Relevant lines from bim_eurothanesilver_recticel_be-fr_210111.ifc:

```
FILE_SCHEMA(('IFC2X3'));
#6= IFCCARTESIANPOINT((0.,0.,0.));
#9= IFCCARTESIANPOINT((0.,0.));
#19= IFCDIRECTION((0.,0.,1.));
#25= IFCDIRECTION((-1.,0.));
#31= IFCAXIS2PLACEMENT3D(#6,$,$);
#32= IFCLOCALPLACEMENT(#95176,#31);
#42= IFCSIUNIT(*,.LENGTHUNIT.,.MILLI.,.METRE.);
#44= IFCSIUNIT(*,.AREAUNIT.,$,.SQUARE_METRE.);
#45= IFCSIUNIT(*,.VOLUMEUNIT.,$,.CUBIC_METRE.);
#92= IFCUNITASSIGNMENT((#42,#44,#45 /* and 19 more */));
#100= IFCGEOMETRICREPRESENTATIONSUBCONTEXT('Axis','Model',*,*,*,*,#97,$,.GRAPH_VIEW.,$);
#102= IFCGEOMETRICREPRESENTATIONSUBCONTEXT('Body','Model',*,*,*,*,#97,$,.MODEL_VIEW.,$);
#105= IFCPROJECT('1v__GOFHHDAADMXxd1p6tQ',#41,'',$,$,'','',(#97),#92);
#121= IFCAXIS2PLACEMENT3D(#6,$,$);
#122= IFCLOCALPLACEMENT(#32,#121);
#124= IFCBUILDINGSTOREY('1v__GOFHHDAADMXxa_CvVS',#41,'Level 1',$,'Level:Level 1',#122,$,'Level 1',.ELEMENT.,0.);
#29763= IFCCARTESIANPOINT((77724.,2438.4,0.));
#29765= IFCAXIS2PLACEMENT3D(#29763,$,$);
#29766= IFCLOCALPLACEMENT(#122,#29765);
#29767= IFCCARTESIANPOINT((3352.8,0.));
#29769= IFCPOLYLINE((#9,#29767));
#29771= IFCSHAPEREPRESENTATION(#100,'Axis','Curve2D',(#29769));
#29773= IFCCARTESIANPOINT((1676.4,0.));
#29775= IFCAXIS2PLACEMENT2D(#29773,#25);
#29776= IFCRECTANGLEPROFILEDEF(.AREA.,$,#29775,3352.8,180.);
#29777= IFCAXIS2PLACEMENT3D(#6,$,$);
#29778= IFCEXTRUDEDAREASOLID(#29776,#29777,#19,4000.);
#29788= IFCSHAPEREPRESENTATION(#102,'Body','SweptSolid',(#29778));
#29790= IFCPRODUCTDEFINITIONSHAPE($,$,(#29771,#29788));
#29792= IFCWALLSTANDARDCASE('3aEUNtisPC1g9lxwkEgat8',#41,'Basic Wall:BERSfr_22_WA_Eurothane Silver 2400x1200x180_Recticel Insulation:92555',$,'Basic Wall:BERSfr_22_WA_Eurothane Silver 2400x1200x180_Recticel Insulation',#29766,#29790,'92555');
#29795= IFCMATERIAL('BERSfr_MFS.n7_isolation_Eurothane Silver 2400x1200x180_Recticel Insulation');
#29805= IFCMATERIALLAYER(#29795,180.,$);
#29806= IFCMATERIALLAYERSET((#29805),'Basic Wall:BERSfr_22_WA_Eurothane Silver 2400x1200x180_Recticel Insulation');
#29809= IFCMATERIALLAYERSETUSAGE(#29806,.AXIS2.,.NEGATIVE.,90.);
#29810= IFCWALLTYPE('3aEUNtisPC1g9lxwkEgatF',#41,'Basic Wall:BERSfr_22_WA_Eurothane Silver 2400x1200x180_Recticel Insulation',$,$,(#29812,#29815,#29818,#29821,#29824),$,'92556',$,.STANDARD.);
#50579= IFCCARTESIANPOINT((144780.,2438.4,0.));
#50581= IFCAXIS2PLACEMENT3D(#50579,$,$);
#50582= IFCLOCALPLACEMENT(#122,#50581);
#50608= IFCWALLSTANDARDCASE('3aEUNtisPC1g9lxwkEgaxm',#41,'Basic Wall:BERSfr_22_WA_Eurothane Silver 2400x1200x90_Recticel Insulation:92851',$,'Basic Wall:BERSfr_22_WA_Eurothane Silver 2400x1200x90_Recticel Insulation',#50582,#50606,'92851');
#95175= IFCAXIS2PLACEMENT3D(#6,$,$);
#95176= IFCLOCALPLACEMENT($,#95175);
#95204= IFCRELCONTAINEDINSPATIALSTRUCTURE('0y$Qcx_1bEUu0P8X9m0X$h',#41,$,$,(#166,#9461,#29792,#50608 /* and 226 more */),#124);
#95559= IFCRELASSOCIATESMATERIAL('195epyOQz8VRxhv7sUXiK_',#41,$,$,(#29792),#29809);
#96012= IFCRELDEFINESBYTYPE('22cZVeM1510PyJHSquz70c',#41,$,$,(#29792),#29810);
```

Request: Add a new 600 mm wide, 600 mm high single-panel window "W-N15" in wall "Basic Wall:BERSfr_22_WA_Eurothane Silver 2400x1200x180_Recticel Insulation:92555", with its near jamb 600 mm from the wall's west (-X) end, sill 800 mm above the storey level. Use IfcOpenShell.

```python
import numpy as np
import ifcopenshell
import ifcopenshell.api.feature
import ifcopenshell.api.geometry
import ifcopenshell.api.root
import ifcopenshell.api.spatial
import ifcopenshell.api.type
import ifcopenshell.geom
import ifcopenshell.util.element
import ifcopenshell.util.placement
import ifcopenshell.util.representation
import ifcopenshell.util.shape
import ifcopenshell.util.unit

model = ifcopenshell.open("bim_eurothanesilver_recticel_be-fr_210111.ifc")
unit_scale = ifcopenshell.util.unit.calculate_unit_scale(model)
settings = ifcopenshell.geom.settings()


def volume(element):
    """Net volume in cubic metres, openings subtracted."""
    shape = ifcopenshell.geom.create_shape(settings, element)
    return ifcopenshell.util.shape.get_volume(shape.geometry)


wall = model.by_guid("3aEUNtisPC1g9lxwkEgat8")
storey = ifcopenshell.util.element.get_container(wall, ifc_class="IfcBuildingStorey")
context = ifcopenshell.util.representation.get_context(model, "Model", "Body", "MODEL_VIEW")
before = volume(wall)

width, height, from_end, sill = 0.6, 0.6, 0.6, 0.8  # metres

# The wall runs along its own X axis, and the end named is its -X end.
wall_shape = ifcopenshell.geom.create_shape(settings, wall)
x, y, z = ifcopenshell.util.shape.get_vertices(wall_shape.geometry).T
start = x.min() + from_end
face, thickness = float(y.min()), float(y.max() - y.min())
wall_matrix = ifcopenshell.util.placement.get_local_placement(wall.ObjectPlacement)
level = ifcopenshell.util.placement.get_local_placement(storey.ObjectPlacement)[2, 3]


def in_wall(x, y):
    """Placement at x, y metres in the wall's axes, at sill height."""
    matrix = wall_matrix.copy()
    matrix[:, 3] = wall_matrix @ np.array([x / unit_scale, y / unit_scale, 0.0, 1.0])
    matrix[2, 3] = level + sill / unit_scale
    return matrix


# Opening: a box that overshoots both wall faces by 50 mm.
opening = ifcopenshell.api.root.create_entity(model, ifc_class="IfcOpeningElement")
box = ifcopenshell.api.geometry.add_wall_representation(
    model, context=context, length=width, height=height, thickness=thickness + 0.1
)
ifcopenshell.api.geometry.assign_representation(model, product=opening, representation=box)
ifcopenshell.api.geometry.edit_object_placement(model, product=opening, matrix=in_wall(start, face - 0.05), is_si=False)
ifcopenshell.api.feature.add_feature(model, feature=opening, element=wall)

window = ifcopenshell.api.root.create_entity(model, ifc_class="IfcWindow", name="W-N15")
window.OverallWidth, window.OverallHeight = width / unit_scale, height / unit_scale
body = ifcopenshell.api.geometry.add_window_representation(
    model,
    context=context,
    overall_width=window.OverallWidth,
    overall_height=window.OverallHeight,
    partition_type="SINGLE_PANEL",
)
ifcopenshell.api.geometry.assign_representation(model, product=window, representation=body)
ifcopenshell.api.spatial.assign_container(model, products=[window], relating_structure=storey)
fills = ifcopenshell.api.feature.add_filling(model, opening=opening, element=window)
fills.OwnerHistory = window.OwnerHistory  # required in IFC2X3

# IFC2X3 keeps the operation on the window style.
style = ifcopenshell.api.root.create_entity(model, ifc_class="IfcWindowStyle", name="W-N15")
style.OperationType, style.ConstructionType = "SINGLE_PANEL", "NOTDEFINED"
style.ParameterTakesPrecedence = style.Sizeable = False
ifcopenshell.api.type.assign_type(model, related_objects=[window], relating_type=style)

# Centre the window in the wall's thickness.
ifcopenshell.api.geometry.edit_object_placement(model, product=window, matrix=in_wall(start, face), is_si=False)
window_shape = ifcopenshell.geom.create_shape(settings, window)
depth = ifcopenshell.util.shape.get_vertices(window_shape.geometry)[:, 1]
offset = face + thickness / 2 - (depth.min() + depth.max()) / 2
ifcopenshell.api.geometry.edit_object_placement(model, product=window, matrix=in_wall(start, offset), is_si=False)

after = volume(wall)

print(f"wall volume {before:.3f} -> {after:.3f} m3")

model.write("bim_eurothanesilver_recticel_be-fr_210111-out.ifc")
```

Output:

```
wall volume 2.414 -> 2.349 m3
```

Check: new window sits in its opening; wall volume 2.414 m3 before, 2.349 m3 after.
